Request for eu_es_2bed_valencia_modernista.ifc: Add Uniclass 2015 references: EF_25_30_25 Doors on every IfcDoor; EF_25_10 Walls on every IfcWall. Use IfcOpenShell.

First a look at what the model holds.

```python
import ifcopenshell

model = ifcopenshell.open("eu_es_2bed_valencia_modernista.ifc")
print(model.schema)
print("classifications:", [c.Name for c in model.by_type("IfcClassification")])
for ifc_class in ("IfcDoor", "IfcRoof", "IfcStair", "IfcWall", "IfcWindow"):
    print(ifc_class, len(model.by_type(ifc_class)))
```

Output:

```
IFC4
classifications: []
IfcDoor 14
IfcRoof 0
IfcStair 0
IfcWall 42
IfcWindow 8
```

```python
import ifcopenshell
import ifcopenshell.api.classification

model = ifcopenshell.open("eu_es_2bed_valencia_modernista.ifc")

system = ifcopenshell.api.classification.add_classification(model, classification="Uniclass 2015")

codes = {
    "IfcDoor": ("EF_25_30_25", "Doors"),
    "IfcWall": ("EF_25_10", "Walls"),
}
for ifc_class, (code, name) in codes.items():
    products = model.by_type(ifc_class)
    ifcopenshell.api.classification.add_reference(
        model, products=products, classification=system, identification=code, name=name
    )
    print(code, len(products))

model.write("eu_es_2bed_valencia_modernista_edited.ifc")
```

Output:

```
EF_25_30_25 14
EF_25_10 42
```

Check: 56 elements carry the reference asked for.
